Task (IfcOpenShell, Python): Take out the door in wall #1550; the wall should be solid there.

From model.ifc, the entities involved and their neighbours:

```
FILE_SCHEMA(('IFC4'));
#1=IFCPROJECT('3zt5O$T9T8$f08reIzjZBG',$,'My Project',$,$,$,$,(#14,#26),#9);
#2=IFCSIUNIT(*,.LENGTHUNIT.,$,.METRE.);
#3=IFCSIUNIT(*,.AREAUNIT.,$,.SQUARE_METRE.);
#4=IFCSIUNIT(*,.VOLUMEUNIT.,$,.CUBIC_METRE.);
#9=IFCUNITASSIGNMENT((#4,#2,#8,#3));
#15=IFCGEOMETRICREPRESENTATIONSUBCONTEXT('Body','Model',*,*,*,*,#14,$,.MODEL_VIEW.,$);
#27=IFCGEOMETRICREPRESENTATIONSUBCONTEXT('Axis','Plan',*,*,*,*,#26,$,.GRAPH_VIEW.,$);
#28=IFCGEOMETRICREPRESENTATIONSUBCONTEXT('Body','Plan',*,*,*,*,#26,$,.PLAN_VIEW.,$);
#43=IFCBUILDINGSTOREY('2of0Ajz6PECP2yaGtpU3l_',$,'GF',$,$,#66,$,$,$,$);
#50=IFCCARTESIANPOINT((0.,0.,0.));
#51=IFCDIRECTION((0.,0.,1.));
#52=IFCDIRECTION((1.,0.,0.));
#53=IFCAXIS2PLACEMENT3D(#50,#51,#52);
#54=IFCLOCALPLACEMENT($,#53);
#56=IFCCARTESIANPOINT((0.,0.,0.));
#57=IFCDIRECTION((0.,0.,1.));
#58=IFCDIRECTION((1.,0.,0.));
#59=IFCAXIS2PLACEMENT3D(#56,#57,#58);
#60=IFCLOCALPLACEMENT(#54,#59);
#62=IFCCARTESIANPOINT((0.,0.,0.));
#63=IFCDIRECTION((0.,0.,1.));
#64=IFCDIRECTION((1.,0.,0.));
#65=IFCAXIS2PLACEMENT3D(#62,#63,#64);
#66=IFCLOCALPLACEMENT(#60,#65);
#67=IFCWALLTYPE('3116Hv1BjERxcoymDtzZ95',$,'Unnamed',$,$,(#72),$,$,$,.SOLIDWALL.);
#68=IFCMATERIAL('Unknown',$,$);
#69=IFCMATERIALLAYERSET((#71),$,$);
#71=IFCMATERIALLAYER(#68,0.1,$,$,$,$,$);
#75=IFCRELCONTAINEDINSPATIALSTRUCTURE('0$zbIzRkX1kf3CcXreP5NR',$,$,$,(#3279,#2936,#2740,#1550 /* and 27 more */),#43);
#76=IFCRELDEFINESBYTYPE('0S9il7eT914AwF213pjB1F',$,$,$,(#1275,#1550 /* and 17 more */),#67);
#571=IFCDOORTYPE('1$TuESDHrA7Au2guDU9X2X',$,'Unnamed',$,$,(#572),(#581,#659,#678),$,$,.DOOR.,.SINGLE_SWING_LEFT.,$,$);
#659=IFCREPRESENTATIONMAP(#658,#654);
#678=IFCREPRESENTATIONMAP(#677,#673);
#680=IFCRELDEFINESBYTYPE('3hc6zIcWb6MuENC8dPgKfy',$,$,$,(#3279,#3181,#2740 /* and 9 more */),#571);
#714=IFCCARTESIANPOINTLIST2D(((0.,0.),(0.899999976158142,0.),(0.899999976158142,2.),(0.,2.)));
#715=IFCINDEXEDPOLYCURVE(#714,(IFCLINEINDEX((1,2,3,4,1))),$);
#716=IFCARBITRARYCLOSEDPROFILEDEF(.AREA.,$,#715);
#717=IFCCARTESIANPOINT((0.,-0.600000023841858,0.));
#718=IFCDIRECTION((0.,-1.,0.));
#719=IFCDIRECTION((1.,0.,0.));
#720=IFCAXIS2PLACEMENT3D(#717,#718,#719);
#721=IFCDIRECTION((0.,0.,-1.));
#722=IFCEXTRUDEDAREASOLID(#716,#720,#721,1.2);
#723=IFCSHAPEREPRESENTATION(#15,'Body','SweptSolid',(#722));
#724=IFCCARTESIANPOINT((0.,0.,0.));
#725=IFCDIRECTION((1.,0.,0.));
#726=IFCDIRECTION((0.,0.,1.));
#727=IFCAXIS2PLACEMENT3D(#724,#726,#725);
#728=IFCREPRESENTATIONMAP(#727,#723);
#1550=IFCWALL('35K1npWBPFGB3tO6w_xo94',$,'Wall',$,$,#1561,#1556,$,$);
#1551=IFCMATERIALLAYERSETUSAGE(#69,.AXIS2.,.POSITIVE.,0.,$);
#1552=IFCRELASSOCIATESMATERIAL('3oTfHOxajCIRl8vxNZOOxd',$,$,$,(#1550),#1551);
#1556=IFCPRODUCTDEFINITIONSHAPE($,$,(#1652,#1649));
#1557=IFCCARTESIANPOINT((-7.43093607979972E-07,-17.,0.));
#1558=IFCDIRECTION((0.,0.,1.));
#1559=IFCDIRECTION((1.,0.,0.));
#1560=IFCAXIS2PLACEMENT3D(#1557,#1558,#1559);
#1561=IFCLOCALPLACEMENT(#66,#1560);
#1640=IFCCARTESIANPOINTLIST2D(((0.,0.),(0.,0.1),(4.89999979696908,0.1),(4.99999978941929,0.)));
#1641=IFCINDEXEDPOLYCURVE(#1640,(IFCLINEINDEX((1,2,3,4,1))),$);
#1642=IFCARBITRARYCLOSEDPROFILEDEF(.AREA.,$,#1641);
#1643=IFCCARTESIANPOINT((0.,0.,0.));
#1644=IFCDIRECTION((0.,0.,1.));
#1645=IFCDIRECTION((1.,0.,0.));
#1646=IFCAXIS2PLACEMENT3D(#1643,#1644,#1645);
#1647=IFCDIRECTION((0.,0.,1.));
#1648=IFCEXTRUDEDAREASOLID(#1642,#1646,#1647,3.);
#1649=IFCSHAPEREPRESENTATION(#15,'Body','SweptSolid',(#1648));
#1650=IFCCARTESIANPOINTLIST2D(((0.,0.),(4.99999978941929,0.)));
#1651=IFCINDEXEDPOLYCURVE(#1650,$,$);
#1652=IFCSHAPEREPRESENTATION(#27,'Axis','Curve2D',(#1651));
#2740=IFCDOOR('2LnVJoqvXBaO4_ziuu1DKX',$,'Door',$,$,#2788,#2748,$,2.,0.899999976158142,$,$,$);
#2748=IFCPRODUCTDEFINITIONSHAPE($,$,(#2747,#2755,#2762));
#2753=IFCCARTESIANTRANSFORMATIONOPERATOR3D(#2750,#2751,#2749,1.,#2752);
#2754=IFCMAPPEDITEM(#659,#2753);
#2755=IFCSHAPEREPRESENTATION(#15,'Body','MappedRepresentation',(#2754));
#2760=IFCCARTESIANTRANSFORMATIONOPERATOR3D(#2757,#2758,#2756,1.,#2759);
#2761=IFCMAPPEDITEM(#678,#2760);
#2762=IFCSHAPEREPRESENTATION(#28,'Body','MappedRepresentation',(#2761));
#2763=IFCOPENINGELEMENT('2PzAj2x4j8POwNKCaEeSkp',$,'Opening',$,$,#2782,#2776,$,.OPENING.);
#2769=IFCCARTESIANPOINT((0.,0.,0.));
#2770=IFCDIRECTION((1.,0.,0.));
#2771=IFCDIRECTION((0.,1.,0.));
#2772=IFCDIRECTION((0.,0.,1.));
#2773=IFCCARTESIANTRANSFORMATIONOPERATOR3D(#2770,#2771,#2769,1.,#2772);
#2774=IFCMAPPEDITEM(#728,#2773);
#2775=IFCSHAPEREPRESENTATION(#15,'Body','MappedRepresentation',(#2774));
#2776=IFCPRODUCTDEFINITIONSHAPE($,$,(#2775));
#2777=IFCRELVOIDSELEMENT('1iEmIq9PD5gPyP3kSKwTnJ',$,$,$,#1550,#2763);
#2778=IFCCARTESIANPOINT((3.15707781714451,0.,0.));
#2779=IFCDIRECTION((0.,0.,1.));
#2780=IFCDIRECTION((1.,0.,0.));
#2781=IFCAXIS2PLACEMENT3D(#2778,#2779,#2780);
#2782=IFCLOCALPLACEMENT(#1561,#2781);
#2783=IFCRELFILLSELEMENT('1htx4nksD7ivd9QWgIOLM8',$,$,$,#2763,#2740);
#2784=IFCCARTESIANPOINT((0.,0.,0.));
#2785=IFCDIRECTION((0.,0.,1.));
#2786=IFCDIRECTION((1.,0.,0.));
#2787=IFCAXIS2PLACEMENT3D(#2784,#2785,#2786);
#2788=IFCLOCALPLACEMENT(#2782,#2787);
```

```python
import ifcopenshell
import ifcopenshell.api.feature
import ifcopenshell.api.root
import ifcopenshell.geom
import ifcopenshell.util.shape

model = ifcopenshell.open("model.ifc")
settings = ifcopenshell.geom.settings()


def volume(element):
    """Net volume in cubic metres, openings subtracted."""
    shape = ifcopenshell.geom.create_shape(settings, element)
    return ifcopenshell.util.shape.get_volume(shape.geometry)


door = model.by_guid("2LnVJoqvXBaO4_ziuu1DKX")
opening = door.FillsVoids[0].RelatingOpeningElement
wall = opening.VoidsElements[0].RelatingBuildingElement
before = volume(wall)

ifcopenshell.api.root.remove_product(model, product=door)
ifcopenshell.api.feature.remove_feature(model, feature=opening)

after = volume(wall)

print(f"wall volume {before:.3f} -> {after:.3f} m3")

model.write("model_updated.ifc")
```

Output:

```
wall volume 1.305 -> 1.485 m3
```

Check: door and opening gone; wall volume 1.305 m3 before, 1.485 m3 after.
